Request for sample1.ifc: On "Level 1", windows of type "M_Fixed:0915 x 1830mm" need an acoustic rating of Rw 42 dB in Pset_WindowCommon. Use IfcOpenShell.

First a look at what the model holds.

```python
import ifcopenshell
import ifcopenshell.util.element

model = ifcopenshell.open("sample1.ifc")
print(model.schema)
storey = next(s for s in model.by_type("IfcBuildingStorey") if s.Name == "Level 1")
windows = [e for e in ifcopenshell.util.element.get_decomposition(storey) if e.is_a("IfcWindow")]
seen = {}
for e in windows:
    element_type = ifcopenshell.util.element.get_type(e)
    key = (element_type.Name if element_type != e and element_type else None, ifcopenshell.util.element.get_pset(e, "Pset_WindowCommon", "AcousticRating"))
    seen[key] = seen.get(key, 0) + 1
for (name, value), count in sorted(seen.items(), key=str):
    print(count, "x", name, "|", value)
```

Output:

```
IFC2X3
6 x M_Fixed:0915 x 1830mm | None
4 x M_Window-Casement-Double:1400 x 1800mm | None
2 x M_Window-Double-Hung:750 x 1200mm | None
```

```python
import ifcopenshell
import ifcopenshell.api.pset
import ifcopenshell.util.element

model = ifcopenshell.open("sample1.ifc")

storey = next(s for s in model.by_type("IfcBuildingStorey") if s.Name == "Level 1")
windows = [e for e in ifcopenshell.util.element.get_decomposition(storey) if e.is_a("IfcWindow")]

count = 0
for e in windows:
    element_type = ifcopenshell.util.element.get_type(e)
    if element_type in (None, e) or element_type.Name != "M_Fixed:0915 x 1830mm":
        continue
    # add_pset returns the element's existing set when there is one.
    pset = ifcopenshell.api.pset.add_pset(model, product=e, name="Pset_WindowCommon")
    ifcopenshell.api.pset.edit_pset(model, pset=pset, properties={"AcousticRating": "Rw 42 dB"})
    count += 1

print(count, "windows updated")

model.write("sample1_v2.ifc")
```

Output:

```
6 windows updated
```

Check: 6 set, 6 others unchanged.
